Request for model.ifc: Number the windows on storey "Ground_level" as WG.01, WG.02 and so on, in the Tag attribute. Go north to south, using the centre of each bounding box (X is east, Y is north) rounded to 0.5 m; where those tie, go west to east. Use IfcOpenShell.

First a look at what the model holds.

```python
import ifcopenshell
import ifcopenshell.util.element
import ifcopenshell.util.placement

model = ifcopenshell.open("model.ifc")
print(model.schema)
storey = next(s for s in model.by_type("IfcBuildingStorey") if s.Name == "Ground_level")
windows = [e for e in ifcopenshell.util.element.get_decomposition(storey) if e.is_a("IfcWindow")]
for e in sorted(windows, key=lambda e: e.id()):
    origin = ifcopenshell.util.placement.get_local_placement(e.ObjectPlacement)[:3, 3]
    print(e.id(), e.Tag, e.Name, origin.round(2) + 0.0, sep=" | ")
```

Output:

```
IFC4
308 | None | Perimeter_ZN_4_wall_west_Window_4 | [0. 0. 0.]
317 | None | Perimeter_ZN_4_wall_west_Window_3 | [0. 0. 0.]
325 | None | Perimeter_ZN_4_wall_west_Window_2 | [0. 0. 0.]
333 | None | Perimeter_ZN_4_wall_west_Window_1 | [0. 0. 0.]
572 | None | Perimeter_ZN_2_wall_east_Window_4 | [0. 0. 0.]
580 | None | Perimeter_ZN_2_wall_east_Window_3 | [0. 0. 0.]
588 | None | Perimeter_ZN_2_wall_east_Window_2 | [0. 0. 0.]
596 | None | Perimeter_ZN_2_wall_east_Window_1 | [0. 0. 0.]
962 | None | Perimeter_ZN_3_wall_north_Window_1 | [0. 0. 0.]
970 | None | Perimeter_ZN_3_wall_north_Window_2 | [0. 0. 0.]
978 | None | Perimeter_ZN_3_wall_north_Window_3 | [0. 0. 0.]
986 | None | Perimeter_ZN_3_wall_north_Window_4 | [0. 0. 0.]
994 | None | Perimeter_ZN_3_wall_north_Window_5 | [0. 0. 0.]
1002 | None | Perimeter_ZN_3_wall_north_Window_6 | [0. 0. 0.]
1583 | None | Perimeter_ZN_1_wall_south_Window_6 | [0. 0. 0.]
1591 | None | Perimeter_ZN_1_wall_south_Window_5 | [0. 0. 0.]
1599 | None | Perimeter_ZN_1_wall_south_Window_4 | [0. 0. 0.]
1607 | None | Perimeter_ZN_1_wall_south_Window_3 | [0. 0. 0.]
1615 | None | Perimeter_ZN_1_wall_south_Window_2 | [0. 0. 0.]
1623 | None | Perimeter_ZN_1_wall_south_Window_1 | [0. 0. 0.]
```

```python
import ifcopenshell
import ifcopenshell.geom
import ifcopenshell.util.element
import ifcopenshell.util.shape

model = ifcopenshell.open("model.ifc")
settings = ifcopenshell.geom.settings()
settings.set("use-world-coords", True)


def centre(element):
    shape = ifcopenshell.geom.create_shape(settings, element)
    return ifcopenshell.util.shape.get_bbox_centroid(shape.geometry)


storey = next(s for s in model.by_type("IfcBuildingStorey") if s.Name == "Ground_level")
windows = [e for e in ifcopenshell.util.element.get_decomposition(storey) if e.is_a("IfcWindow")]

# Insertion points can sit at a corner or the storey origin, so sort by the geometry (in metres).
centres = {e: centre(e) for e in windows}
windows.sort(key=lambda e: (-round(centres[e][1] / 0.5), centres[e][0]))

for i, e in enumerate(windows, start=1):
    number = f"WG.{i:02d}"
    e.Tag = number
    print(e.id(), number)

model.write("model_rev.ifc")
```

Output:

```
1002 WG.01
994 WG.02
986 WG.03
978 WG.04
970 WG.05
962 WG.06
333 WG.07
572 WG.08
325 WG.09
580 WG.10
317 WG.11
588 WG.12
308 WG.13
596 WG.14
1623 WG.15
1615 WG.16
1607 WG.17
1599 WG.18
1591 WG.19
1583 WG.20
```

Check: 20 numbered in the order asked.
